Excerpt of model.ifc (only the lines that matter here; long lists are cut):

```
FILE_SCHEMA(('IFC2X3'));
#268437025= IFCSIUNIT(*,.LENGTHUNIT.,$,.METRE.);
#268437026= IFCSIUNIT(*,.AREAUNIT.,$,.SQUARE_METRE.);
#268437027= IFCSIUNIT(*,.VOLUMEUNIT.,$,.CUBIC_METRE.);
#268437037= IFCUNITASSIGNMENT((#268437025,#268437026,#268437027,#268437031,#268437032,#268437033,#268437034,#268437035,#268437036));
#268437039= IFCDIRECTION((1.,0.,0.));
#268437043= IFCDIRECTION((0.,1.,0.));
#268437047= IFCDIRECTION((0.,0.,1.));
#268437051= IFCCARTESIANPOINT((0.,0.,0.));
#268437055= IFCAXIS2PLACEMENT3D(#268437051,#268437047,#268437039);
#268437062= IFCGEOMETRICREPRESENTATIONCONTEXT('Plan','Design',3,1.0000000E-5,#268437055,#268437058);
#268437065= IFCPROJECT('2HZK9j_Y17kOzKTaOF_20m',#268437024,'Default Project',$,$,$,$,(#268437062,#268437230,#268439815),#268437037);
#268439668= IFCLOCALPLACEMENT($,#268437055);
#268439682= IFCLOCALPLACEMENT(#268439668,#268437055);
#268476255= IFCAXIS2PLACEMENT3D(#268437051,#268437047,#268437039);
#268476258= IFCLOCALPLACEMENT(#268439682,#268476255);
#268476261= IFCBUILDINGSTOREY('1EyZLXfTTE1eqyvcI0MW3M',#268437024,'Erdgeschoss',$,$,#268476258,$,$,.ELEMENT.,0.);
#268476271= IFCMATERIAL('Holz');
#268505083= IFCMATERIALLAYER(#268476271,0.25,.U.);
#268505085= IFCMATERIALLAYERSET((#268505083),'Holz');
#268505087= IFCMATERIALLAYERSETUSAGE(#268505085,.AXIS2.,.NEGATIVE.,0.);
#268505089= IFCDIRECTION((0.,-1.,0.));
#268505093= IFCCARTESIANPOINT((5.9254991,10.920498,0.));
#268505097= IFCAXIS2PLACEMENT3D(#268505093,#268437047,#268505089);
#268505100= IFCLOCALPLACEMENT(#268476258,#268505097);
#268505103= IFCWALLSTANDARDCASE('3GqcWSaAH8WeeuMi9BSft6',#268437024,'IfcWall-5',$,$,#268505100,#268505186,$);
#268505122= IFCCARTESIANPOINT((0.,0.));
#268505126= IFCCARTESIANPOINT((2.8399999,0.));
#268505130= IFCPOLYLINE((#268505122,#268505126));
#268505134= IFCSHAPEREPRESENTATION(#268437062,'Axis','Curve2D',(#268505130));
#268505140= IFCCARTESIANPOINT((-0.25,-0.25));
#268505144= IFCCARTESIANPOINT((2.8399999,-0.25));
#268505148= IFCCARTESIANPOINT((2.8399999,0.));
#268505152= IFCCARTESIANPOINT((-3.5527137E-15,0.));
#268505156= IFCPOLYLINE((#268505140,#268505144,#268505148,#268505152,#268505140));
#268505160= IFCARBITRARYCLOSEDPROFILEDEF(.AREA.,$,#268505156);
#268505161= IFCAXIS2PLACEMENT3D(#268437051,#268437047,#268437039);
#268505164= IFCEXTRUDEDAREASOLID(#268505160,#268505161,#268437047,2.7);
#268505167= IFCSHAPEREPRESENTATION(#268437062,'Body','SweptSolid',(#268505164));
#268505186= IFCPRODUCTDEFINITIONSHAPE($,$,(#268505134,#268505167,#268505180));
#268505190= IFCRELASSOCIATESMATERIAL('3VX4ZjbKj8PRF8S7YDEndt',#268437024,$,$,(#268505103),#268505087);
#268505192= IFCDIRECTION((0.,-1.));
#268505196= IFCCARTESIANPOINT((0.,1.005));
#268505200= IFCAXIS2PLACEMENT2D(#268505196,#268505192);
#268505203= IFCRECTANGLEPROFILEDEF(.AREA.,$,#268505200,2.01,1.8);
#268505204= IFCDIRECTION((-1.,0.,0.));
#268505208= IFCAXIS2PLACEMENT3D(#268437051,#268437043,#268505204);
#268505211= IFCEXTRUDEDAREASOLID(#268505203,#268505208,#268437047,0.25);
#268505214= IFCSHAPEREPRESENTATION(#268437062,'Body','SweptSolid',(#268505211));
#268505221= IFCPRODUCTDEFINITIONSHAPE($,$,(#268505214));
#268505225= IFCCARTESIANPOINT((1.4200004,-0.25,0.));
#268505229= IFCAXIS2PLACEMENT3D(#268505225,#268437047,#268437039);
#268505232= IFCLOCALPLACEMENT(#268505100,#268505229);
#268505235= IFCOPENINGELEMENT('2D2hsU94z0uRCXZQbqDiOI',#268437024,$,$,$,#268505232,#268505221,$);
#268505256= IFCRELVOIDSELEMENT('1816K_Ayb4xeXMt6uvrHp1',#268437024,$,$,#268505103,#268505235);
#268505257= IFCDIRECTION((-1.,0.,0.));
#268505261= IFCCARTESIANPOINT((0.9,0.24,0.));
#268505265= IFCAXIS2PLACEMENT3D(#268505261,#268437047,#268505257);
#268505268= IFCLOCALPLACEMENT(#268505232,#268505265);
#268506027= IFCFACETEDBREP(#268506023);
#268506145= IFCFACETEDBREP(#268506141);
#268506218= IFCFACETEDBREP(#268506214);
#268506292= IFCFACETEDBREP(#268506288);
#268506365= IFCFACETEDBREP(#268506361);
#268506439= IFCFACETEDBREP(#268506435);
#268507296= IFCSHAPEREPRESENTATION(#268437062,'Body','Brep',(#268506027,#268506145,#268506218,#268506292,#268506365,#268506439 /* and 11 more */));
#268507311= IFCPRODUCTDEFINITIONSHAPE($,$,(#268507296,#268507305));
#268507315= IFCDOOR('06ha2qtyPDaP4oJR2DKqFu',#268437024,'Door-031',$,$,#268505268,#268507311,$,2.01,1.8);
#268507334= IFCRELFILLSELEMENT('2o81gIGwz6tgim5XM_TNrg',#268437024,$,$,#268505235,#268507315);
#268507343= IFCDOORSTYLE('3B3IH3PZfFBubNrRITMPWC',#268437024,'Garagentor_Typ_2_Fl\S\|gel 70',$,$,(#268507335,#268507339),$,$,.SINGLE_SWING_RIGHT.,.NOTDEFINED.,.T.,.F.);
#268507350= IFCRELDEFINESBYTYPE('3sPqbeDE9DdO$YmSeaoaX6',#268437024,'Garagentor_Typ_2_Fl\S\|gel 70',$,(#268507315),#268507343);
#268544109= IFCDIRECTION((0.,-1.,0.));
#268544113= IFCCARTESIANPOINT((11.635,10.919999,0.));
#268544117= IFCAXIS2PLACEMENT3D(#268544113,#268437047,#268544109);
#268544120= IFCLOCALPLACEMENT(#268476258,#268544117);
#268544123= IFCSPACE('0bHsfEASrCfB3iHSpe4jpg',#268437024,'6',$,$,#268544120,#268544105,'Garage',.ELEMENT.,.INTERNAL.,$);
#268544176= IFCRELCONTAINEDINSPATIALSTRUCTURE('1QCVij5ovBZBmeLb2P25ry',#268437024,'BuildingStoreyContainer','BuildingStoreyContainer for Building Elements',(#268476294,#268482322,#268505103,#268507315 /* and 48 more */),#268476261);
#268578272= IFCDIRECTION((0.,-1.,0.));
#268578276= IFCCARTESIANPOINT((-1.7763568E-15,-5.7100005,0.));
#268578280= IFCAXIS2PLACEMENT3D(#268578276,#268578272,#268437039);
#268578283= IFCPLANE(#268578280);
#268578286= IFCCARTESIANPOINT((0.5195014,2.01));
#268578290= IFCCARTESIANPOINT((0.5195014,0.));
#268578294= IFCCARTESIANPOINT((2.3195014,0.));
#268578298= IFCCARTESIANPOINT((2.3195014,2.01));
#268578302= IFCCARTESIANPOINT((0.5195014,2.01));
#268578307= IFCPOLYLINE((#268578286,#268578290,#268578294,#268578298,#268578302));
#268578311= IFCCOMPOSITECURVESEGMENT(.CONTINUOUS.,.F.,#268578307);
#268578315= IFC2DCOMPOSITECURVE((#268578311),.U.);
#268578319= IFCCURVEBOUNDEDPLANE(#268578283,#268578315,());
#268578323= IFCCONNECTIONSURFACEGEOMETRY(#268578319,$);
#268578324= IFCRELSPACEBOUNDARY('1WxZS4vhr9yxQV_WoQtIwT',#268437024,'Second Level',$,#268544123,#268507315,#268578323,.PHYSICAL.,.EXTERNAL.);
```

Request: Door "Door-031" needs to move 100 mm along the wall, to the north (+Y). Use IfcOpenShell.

```python
import numpy as np
import ifcopenshell
import ifcopenshell.api.geometry
import ifcopenshell.util.placement

model = ifcopenshell.open("model.ifc")

door = model.by_id(268507315)
opening = door.FillsVoids[0].RelatingOpeningElement
wall = opening.VoidsElements[0].RelatingBuildingElement

wall_matrix = ifcopenshell.util.placement.get_local_placement(wall.ObjectPlacement)
shift = wall_matrix[:3, 0] * -0.1
before = ifcopenshell.util.placement.get_local_placement(door.ObjectPlacement)[:3, 3].copy()

# The door is placed relative to its opening, so it follows when the opening moves.
matrix = ifcopenshell.util.placement.get_local_placement(opening.ObjectPlacement)
matrix[:3, 3] += shift
ifcopenshell.api.geometry.edit_object_placement(
    model, product=opening, matrix=matrix, is_si=False, should_transform_children=True
)

# Space boundary surfaces are stored in each space's coordinates; move them too.
for rel in door.ProvidesBoundaries:
    if not rel.ConnectionGeometry:
        continue
    surface = rel.ConnectionGeometry.SurfaceOnRelatingElement.BasisSurface
    space_matrix = ifcopenshell.util.placement.get_local_placement(rel.RelatingSpace.ObjectPlacement)
    point = np.array(surface.Position.Location.Coordinates) + space_matrix[:3, :3].T @ shift
    surface.Position = model.createIfcAxis2Placement3D(
        model.createIfcCartesianPoint(point.tolist()), surface.Position.Axis, surface.Position.RefDirection
    )

after = ifcopenshell.util.placement.get_local_placement(door.ObjectPlacement)[:3, 3]
print("door moved by", (after - before).round(3) + 0.0)

model.write("model-out.ifc")
```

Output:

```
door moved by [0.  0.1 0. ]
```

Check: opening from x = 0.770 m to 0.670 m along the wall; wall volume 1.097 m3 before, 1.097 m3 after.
